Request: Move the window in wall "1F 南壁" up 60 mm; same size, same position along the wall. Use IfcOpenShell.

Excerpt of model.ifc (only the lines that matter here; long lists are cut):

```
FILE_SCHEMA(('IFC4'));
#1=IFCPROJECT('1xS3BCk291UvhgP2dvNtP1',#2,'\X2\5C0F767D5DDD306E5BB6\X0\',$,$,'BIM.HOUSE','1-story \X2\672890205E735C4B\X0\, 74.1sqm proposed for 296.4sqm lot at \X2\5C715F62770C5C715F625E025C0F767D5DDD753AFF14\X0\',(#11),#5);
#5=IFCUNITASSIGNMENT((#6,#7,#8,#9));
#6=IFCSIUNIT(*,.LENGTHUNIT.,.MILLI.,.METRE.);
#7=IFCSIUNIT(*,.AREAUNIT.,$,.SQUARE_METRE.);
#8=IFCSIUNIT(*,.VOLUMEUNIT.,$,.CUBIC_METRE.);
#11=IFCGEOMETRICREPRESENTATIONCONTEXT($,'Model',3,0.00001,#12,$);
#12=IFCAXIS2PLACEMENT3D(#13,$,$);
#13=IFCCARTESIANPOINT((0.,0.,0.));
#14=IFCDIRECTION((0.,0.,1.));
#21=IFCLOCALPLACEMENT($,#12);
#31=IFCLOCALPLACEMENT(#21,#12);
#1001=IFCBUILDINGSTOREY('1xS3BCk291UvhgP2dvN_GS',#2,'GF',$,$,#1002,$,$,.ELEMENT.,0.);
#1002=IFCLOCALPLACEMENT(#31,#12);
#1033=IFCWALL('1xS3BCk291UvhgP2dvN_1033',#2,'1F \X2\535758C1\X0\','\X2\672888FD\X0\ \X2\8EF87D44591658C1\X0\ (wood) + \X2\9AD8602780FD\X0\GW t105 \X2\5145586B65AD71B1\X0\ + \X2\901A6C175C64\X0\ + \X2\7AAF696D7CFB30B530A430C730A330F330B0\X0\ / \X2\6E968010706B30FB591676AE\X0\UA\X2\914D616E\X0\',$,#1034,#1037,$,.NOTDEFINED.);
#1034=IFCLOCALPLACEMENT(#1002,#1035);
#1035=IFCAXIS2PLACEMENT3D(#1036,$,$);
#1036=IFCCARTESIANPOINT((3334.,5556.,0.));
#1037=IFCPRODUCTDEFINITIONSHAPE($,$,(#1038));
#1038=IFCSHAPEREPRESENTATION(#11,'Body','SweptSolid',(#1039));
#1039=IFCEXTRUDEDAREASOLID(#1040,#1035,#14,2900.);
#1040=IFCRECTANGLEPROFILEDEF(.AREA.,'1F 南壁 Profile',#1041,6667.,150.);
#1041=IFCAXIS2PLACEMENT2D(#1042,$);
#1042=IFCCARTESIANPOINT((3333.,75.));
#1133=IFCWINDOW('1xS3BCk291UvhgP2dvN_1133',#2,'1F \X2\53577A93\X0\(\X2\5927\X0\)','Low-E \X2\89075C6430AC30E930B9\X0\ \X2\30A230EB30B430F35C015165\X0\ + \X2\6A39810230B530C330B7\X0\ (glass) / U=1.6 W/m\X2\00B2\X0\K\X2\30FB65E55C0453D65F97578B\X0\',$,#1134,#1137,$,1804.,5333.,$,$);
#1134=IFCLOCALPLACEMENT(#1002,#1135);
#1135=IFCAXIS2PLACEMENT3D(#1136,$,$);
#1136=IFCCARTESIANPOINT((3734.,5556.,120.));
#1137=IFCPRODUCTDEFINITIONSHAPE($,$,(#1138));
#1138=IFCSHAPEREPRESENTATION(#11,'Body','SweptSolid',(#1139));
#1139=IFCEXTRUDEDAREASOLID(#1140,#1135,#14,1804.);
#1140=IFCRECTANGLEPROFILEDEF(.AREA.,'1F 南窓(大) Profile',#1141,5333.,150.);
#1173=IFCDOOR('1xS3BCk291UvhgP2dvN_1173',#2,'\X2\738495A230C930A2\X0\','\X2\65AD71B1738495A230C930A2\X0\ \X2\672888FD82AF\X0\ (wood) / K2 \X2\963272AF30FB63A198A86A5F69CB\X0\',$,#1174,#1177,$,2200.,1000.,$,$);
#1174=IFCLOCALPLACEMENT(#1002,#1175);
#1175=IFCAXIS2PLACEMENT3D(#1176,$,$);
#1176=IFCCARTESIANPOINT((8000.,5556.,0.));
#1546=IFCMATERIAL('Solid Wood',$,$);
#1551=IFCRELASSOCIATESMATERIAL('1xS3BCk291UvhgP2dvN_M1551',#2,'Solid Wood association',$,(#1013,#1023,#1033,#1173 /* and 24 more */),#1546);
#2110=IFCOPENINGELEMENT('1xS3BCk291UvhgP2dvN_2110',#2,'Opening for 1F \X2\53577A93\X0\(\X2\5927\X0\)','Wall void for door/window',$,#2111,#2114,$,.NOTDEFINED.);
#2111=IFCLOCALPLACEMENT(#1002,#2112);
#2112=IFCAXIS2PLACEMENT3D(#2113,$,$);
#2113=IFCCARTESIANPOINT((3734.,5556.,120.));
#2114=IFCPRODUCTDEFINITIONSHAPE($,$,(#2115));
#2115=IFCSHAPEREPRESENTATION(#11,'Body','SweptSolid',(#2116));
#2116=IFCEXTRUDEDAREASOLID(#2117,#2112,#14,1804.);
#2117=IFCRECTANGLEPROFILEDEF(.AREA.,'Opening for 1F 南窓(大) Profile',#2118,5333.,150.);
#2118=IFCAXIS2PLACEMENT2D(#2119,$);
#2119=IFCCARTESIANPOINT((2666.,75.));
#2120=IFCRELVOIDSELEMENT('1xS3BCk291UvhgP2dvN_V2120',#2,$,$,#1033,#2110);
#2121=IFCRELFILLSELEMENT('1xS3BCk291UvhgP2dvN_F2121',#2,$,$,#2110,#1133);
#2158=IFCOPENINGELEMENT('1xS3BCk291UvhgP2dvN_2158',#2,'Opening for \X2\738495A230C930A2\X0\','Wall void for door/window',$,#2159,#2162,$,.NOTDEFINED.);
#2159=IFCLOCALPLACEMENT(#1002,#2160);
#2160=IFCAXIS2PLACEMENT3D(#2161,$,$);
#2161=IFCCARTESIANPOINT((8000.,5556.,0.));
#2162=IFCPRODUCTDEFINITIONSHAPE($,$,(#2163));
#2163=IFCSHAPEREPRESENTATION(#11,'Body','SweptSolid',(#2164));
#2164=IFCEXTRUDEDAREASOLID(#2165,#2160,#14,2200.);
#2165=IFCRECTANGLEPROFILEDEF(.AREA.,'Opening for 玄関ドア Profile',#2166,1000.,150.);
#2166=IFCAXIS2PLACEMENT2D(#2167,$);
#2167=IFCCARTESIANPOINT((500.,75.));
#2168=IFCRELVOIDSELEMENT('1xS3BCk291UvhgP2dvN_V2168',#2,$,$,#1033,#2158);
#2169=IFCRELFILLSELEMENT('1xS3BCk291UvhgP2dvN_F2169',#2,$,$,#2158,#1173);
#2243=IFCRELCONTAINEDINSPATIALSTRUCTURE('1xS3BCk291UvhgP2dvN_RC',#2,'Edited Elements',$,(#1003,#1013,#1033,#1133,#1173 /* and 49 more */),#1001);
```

```python
import numpy as np
import ifcopenshell
import ifcopenshell.api.geometry
import ifcopenshell.util.placement
import ifcopenshell.util.unit

model = ifcopenshell.open("model.ifc")
unit_scale = ifcopenshell.util.unit.calculate_unit_scale(model)

window = model.by_guid("1xS3BCk291UvhgP2dvN_1133")
opening = window.FillsVoids[0].RelatingOpeningElement
dz = 0.06 / unit_scale

shift = np.array([0.0, 0.0, dz])
# The window is not placed relative to its opening, so move both.
for product in (opening, window):
    matrix = ifcopenshell.util.placement.get_local_placement(product.ObjectPlacement)
    matrix[:3, 3] += shift
    ifcopenshell.api.geometry.edit_object_placement(model, product=product, matrix=matrix, is_si=False)

print(f"moved by {dz * unit_scale:+.3f} m")

model.write("model_edited.ifc")
```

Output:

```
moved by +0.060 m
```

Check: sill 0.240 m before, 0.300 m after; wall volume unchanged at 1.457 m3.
